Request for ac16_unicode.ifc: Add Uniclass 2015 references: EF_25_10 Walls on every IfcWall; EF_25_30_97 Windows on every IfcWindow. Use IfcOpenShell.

First a look at what the model holds.

```python
import ifcopenshell

model = ifcopenshell.open("ac16_unicode.ifc")
print(model.schema)
print("classifications:", [c.Name for c in model.by_type("IfcClassification")])
for ifc_class in ("IfcDoor", "IfcRoof", "IfcStair", "IfcWall", "IfcWindow"):
    print(ifc_class, len(model.by_type(ifc_class)))
```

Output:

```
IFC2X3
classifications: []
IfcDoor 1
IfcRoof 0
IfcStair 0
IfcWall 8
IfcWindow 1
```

```python
import ifcopenshell
import ifcopenshell.api.classification

model = ifcopenshell.open("ac16_unicode.ifc")

# IFC2X3 requires Source and Edition and has no link from the project to the system.
system = model.create_entity("IfcClassification", Source="NBS", Edition="2015", Name="Uniclass 2015")

codes = {
    "IfcWall": ("EF_25_10", "Walls"),
    "IfcWindow": ("EF_25_30_97", "Windows"),
}
for ifc_class, (code, name) in codes.items():
    products = model.by_type(ifc_class)
    ifcopenshell.api.classification.add_reference(
        model, products=products, classification=system, identification=code, name=name
    )
    print(code, len(products))

model.write("ac16_unicode_v2.ifc")
```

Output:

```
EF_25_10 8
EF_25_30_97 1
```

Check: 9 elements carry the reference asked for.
